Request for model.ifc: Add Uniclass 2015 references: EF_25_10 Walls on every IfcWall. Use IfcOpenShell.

First a look at what the model holds.

```python
import ifcopenshell

model = ifcopenshell.open("model.ifc")
print(model.schema)
print("classifications:", [c.Name for c in model.by_type("IfcClassification")])
for ifc_class in ("IfcDoor", "IfcRoof", "IfcStair", "IfcWall", "IfcWindow"):
    print(ifc_class, len(model.by_type(ifc_class)))
```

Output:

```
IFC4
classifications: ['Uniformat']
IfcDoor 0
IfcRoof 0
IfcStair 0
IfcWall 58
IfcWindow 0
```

```python
import ifcopenshell
import ifcopenshell.api.classification

model = ifcopenshell.open("model.ifc")

system = ifcopenshell.api.classification.add_classification(model, classification="Uniclass 2015")

codes = {
    "IfcWall": ("EF_25_10", "Walls"),
}
for ifc_class, (code, name) in codes.items():
    products = model.by_type(ifc_class)
    ifcopenshell.api.classification.add_reference(
        model, products=products, classification=system, identification=code, name=name
    )
    print(code, len(products))

model.write("model-out.ifc")
```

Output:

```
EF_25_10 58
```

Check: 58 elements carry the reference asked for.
